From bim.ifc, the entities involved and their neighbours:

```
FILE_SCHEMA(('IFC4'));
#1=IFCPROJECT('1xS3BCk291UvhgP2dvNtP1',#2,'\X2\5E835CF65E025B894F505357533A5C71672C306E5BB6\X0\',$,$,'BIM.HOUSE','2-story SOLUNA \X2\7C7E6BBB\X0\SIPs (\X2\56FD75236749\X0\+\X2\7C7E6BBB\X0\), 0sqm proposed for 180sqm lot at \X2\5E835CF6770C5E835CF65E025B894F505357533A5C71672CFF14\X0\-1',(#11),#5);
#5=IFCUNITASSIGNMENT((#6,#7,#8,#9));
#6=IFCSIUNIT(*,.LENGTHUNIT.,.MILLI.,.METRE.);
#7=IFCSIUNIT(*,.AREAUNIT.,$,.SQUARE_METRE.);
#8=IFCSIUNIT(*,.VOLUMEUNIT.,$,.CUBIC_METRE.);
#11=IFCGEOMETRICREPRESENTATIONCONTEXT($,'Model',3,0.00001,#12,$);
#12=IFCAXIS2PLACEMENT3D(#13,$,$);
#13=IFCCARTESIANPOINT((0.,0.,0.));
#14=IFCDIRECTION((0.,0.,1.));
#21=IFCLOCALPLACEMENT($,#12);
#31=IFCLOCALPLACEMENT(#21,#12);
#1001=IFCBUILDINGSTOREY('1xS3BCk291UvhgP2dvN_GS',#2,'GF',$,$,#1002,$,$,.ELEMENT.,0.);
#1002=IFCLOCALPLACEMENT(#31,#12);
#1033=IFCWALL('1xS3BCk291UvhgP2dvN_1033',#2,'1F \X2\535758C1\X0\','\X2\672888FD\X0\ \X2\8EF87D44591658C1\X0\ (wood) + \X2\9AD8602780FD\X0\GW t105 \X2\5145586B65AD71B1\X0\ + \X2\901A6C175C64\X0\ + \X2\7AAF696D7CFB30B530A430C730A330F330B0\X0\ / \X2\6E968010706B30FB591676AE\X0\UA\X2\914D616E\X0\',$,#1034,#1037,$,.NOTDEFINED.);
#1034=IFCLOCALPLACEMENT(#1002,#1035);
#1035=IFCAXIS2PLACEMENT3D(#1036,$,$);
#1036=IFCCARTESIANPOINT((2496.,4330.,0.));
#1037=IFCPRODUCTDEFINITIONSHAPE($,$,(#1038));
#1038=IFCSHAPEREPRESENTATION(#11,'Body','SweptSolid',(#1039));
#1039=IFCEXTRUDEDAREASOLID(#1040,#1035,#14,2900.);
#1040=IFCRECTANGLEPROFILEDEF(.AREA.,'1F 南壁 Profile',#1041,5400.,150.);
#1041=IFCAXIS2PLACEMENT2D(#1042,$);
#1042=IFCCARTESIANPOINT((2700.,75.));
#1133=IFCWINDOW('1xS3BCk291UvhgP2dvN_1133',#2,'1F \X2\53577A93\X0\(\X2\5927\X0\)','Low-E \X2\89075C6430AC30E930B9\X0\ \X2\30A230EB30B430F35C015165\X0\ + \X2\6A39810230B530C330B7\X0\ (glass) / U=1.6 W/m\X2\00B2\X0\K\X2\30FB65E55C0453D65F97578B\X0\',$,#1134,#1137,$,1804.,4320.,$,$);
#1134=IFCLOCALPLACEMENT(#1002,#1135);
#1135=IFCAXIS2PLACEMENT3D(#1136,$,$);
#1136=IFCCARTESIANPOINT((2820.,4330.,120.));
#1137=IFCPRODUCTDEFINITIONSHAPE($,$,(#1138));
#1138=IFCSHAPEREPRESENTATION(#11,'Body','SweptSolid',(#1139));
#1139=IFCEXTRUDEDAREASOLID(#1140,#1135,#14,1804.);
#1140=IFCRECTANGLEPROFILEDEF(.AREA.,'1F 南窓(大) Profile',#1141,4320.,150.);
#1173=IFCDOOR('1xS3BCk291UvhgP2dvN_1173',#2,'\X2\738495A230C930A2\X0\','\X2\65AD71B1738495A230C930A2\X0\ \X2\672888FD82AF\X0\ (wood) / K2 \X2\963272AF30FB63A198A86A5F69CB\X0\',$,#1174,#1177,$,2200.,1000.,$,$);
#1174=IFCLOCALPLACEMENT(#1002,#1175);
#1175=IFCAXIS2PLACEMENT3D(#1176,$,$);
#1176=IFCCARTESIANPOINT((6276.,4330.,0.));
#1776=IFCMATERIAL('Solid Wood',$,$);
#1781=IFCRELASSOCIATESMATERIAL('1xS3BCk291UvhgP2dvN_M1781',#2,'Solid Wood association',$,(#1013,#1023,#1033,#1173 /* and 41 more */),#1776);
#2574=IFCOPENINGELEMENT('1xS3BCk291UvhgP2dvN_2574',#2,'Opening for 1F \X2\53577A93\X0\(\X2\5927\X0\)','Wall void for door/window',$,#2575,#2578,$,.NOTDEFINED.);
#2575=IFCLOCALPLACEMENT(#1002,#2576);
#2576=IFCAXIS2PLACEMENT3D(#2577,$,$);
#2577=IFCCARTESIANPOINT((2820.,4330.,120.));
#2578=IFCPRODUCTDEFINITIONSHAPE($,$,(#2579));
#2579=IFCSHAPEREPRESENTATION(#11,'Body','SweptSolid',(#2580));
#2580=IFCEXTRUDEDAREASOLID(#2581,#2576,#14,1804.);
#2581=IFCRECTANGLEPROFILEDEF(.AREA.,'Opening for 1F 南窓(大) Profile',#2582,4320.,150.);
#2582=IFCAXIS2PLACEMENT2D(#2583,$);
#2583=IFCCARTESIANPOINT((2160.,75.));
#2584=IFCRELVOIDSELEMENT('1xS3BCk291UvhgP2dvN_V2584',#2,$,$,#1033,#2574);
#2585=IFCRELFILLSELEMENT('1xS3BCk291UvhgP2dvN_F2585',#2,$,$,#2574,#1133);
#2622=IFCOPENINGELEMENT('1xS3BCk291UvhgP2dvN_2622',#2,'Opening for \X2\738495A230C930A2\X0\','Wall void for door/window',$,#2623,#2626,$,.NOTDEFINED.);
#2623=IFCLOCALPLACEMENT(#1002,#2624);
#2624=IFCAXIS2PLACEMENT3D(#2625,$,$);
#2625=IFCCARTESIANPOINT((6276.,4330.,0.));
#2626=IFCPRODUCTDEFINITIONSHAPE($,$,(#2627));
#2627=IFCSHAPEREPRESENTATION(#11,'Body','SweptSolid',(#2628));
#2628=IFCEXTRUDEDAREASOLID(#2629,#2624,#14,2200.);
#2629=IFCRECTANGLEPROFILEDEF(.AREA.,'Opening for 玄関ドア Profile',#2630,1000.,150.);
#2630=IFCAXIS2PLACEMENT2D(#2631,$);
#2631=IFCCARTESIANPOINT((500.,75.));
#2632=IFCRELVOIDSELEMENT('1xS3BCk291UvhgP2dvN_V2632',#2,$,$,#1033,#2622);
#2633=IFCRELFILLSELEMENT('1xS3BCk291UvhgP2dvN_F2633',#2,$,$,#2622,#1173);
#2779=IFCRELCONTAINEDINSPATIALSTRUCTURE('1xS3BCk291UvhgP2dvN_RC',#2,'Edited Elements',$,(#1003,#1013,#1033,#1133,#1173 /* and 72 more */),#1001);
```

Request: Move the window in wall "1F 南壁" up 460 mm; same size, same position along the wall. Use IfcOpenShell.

```python
import numpy as np
import ifcopenshell
import ifcopenshell.api.geometry
import ifcopenshell.util.placement
import ifcopenshell.util.unit

model = ifcopenshell.open("bim.ifc")
unit_scale = ifcopenshell.util.unit.calculate_unit_scale(model)

window = model.by_guid("1xS3BCk291UvhgP2dvN_1133")
opening = window.FillsVoids[0].RelatingOpeningElement
dz = 0.46 / unit_scale

shift = np.array([0.0, 0.0, dz])
# The window is not placed relative to its opening, so move both.
for product in (opening, window):
    matrix = ifcopenshell.util.placement.get_local_placement(product.ObjectPlacement)
    matrix[:3, 3] += shift
    ifcopenshell.api.geometry.edit_object_placement(model, product=product, matrix=matrix, is_si=False)

print(f"moved by {dz * unit_scale:+.3f} m")

model.write("bim_updated.ifc")
```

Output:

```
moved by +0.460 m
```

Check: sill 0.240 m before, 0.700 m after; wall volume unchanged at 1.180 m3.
